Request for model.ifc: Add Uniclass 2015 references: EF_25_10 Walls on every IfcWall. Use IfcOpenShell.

First a look at what the model holds.

```python
import ifcopenshell

model = ifcopenshell.open("model.ifc")
print(model.schema)
print("classifications:", [c.Name for c in model.by_type("IfcClassification")])
for ifc_class in ("IfcDoor", "IfcRoof", "IfcStair", "IfcWall", "IfcWindow"):
    print(ifc_class, len(model.by_type(ifc_class)))
```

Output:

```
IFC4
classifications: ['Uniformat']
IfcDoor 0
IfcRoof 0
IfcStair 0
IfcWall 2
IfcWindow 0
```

```python
import ifcopenshell
import ifcopenshell.api.classification

model = ifcopenshell.open("model.ifc")

system = ifcopenshell.api.classification.add_classification(model, classification="Uniclass 2015")

codes = {
    "IfcWall": ("EF_25_10", "Walls"),
}
for ifc_class, (code, name) in codes.items():
    products = model.by_type(ifc_class)
    ifcopenshell.api.classification.add_reference(
        model, products=products, classification=system, identification=code, name=name
    )
    print(code, len(products))

model.write("model_updated.ifc")
```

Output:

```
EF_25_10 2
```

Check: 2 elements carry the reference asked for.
